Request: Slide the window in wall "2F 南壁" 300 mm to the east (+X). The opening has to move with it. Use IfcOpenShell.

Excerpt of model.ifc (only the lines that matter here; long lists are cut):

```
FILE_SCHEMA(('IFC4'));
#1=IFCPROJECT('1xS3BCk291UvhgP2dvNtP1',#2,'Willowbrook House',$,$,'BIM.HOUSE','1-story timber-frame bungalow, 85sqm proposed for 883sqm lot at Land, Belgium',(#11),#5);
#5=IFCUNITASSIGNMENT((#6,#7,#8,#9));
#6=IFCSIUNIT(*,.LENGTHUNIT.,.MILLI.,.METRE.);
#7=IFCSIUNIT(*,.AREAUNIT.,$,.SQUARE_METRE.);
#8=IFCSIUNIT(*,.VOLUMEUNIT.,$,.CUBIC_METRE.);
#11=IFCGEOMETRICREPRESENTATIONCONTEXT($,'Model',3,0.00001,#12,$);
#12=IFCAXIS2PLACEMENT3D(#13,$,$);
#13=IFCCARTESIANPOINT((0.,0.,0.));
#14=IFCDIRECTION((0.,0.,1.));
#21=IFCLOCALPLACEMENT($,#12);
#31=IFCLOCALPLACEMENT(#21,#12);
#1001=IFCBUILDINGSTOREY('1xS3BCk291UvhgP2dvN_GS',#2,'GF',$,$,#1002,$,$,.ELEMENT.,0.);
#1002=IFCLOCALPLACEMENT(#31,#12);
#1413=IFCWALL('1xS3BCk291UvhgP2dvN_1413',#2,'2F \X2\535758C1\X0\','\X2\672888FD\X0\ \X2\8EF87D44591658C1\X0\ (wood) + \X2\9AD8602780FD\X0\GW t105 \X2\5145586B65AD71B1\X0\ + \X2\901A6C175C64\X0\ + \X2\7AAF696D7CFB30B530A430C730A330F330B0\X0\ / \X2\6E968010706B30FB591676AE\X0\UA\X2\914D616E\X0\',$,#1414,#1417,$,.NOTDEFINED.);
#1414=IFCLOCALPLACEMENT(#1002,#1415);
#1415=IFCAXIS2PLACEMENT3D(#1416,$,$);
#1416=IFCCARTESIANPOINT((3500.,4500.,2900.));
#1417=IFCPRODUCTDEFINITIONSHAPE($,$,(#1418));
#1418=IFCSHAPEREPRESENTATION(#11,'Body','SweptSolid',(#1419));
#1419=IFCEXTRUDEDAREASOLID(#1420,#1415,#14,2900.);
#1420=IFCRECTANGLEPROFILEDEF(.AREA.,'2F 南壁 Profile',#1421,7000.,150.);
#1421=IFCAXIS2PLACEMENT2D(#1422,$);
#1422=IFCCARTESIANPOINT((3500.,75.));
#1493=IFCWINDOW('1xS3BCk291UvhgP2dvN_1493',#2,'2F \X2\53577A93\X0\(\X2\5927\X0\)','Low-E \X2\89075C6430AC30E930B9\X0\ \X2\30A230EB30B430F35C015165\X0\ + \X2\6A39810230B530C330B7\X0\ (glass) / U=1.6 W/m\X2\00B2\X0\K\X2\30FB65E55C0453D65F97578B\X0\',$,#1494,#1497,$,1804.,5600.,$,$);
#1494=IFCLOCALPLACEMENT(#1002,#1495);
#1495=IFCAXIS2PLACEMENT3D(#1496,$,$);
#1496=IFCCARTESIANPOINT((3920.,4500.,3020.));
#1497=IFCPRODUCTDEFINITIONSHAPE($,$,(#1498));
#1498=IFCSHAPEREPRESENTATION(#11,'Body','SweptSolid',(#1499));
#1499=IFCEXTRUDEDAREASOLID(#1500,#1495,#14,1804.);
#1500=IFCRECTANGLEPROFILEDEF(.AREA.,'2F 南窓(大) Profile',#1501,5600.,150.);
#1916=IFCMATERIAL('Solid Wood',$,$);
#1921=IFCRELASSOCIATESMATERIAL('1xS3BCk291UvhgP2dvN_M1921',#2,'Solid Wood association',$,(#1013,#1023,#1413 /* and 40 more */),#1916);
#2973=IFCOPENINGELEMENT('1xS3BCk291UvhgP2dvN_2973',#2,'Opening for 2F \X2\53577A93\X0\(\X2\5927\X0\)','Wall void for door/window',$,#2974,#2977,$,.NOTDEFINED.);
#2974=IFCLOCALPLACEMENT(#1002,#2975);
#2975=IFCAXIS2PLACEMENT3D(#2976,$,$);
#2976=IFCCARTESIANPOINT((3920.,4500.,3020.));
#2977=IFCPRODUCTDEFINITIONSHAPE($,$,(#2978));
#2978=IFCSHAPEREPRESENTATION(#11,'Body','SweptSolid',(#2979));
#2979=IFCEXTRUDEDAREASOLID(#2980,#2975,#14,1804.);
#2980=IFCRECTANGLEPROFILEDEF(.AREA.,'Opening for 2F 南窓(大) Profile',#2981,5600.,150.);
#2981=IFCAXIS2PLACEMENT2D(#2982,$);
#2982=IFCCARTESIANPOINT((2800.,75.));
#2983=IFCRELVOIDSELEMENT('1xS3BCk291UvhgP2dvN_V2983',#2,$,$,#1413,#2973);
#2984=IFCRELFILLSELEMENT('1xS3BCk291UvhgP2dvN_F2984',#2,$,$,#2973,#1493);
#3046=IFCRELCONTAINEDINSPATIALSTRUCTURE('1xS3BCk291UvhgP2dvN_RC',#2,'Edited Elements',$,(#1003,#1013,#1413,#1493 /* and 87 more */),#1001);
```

```python
import ifcopenshell
import ifcopenshell.api.geometry
import ifcopenshell.util.placement
import ifcopenshell.util.unit

model = ifcopenshell.open("model.ifc")
unit_scale = ifcopenshell.util.unit.calculate_unit_scale(model)

window = model.by_guid("1xS3BCk291UvhgP2dvN_1493")
opening = window.FillsVoids[0].RelatingOpeningElement
wall = opening.VoidsElements[0].RelatingBuildingElement

wall_matrix = ifcopenshell.util.placement.get_local_placement(wall.ObjectPlacement)
shift = wall_matrix[:3, 0] * 0.3 / unit_scale
before = ifcopenshell.util.placement.get_local_placement(window.ObjectPlacement)[:3, 3].copy()

# The window is not placed relative to its opening, so move both.
for product in (opening, window):
    matrix = ifcopenshell.util.placement.get_local_placement(product.ObjectPlacement)
    matrix[:3, 3] += shift
    ifcopenshell.api.geometry.edit_object_placement(model, product=product, matrix=matrix, is_si=False)

after = ifcopenshell.util.placement.get_local_placement(window.ObjectPlacement)[:3, 3]
print("window moved by", (after - before).round(3) + 0.0)

model.write("model_rev.ifc")
```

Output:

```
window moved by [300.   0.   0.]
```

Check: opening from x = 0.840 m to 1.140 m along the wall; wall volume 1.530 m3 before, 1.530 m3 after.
